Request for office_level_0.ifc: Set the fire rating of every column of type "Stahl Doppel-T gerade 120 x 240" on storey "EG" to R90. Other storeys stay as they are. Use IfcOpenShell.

First a look at what the model holds.

```python
import ifcopenshell
import ifcopenshell.util.element

model = ifcopenshell.open("office_level_0.ifc")
print(model.schema)
storey = next(s for s in model.by_type("IfcBuildingStorey") if s.Name == "EG")
columns = [e for e in ifcopenshell.util.element.get_decomposition(storey) if e.is_a("IfcColumn")]
seen = {}
for e in columns:
    element_type = ifcopenshell.util.element.get_type(e)
    key = (element_type.Name if element_type != e and element_type else None, ifcopenshell.util.element.get_pset(e, "Pset_ColumnCommon", "FireRating"))
    seen[key] = seen.get(key, 0) + 1
for (name, value), count in sorted(seen.items(), key=str):
    print(count, "x", name, "|", value)
```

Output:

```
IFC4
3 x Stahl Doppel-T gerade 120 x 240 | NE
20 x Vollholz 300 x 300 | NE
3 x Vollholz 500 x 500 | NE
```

```python
import ifcopenshell
import ifcopenshell.api.pset
import ifcopenshell.util.element

model = ifcopenshell.open("office_level_0.ifc")

storey = next(s for s in model.by_type("IfcBuildingStorey") if s.Name == "EG")
columns = [e for e in ifcopenshell.util.element.get_decomposition(storey) if e.is_a("IfcColumn")]

count = 0
for e in columns:
    element_type = ifcopenshell.util.element.get_type(e)
    if element_type in (None, e) or element_type.Name != "Stahl Doppel-T gerade 120 x 240":
        continue
    # add_pset returns the element's existing set when there is one.
    pset = ifcopenshell.api.pset.add_pset(model, product=e, name="Pset_ColumnCommon")
    ifcopenshell.api.pset.edit_pset(model, pset=pset, properties={"FireRating": "R90"})
    count += 1

print(count, "columns updated")

model.write("office_level_0_updated.ifc")
```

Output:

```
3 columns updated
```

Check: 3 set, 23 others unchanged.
